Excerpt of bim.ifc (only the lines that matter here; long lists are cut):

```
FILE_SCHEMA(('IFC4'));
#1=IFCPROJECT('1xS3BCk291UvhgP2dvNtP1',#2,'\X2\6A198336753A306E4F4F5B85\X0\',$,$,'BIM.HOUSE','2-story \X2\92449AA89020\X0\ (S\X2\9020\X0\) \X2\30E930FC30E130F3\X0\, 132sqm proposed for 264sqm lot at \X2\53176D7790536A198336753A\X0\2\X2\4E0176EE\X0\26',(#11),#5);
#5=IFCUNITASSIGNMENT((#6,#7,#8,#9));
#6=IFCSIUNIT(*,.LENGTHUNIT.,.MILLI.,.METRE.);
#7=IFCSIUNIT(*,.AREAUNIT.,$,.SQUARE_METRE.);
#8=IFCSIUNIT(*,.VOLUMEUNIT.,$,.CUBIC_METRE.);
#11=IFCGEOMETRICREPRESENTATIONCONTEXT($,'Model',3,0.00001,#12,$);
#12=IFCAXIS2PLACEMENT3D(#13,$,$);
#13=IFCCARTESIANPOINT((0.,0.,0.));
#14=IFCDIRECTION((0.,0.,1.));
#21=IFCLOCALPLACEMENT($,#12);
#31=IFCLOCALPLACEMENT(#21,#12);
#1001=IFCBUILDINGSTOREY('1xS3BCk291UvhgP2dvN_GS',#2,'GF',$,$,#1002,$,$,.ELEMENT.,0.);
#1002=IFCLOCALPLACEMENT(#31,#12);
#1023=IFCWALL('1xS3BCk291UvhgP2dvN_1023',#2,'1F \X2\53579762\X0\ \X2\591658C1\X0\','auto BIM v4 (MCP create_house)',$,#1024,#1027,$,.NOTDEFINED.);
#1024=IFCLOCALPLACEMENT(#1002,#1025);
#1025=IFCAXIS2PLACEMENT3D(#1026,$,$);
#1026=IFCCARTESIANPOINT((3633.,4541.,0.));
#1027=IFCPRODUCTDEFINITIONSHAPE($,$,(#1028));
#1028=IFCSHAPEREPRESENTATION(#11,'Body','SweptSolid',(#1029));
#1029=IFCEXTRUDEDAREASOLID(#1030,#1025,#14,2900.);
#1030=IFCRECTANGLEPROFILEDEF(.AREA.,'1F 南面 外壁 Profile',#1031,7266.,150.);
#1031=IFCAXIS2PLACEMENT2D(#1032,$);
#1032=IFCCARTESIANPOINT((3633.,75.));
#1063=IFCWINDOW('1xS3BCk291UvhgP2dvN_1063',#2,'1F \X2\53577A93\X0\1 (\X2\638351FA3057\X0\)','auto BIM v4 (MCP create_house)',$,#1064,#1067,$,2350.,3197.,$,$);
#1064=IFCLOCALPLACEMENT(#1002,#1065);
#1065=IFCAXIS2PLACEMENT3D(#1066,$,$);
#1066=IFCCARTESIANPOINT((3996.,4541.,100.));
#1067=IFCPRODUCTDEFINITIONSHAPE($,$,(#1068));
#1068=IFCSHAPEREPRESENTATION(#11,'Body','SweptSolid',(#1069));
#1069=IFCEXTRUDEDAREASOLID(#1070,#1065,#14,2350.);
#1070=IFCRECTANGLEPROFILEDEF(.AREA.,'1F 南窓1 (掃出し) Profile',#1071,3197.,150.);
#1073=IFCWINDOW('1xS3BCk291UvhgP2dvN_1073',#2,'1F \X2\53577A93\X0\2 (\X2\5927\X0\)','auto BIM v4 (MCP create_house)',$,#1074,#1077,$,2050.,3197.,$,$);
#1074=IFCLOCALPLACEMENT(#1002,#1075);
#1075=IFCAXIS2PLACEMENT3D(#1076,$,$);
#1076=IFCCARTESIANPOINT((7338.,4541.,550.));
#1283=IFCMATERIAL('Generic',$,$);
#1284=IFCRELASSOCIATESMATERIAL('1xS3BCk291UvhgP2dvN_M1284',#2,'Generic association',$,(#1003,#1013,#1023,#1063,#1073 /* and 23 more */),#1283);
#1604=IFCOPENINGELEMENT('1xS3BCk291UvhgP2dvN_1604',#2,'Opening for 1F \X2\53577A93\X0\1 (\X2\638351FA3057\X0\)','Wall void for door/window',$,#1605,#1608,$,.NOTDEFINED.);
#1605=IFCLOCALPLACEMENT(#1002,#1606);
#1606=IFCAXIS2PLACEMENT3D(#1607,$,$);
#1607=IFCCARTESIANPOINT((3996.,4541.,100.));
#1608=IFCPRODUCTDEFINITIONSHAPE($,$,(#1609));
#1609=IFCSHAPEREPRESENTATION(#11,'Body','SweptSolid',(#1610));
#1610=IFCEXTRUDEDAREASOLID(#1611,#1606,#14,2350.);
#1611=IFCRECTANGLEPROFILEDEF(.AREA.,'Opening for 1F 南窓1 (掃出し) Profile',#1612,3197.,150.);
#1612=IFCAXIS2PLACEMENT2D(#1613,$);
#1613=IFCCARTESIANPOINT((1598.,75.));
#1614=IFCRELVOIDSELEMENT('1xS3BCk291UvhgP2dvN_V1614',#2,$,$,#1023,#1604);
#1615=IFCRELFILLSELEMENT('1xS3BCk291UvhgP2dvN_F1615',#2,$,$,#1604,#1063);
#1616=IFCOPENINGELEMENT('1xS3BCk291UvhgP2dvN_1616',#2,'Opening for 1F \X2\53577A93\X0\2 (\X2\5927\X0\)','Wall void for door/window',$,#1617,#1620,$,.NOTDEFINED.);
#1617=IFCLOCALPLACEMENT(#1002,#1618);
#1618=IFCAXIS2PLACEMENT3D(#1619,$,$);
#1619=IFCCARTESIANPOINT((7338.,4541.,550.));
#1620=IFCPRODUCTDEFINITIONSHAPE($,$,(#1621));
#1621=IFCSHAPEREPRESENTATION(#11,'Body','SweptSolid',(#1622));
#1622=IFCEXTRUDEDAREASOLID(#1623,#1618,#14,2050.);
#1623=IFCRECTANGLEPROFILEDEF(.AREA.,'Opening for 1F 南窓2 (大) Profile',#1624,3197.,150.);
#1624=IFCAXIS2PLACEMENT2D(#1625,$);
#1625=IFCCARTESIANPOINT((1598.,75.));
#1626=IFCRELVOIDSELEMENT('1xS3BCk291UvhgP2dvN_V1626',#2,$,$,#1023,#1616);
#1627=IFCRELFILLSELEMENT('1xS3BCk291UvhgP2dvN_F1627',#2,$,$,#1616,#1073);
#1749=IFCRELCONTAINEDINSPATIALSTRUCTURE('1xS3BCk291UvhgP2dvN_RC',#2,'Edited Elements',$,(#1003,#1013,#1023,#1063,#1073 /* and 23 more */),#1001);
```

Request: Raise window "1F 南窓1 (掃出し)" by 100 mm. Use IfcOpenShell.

```python
import numpy as np
import ifcopenshell
import ifcopenshell.api.geometry
import ifcopenshell.util.placement
import ifcopenshell.util.unit

model = ifcopenshell.open("bim.ifc")
unit_scale = ifcopenshell.util.unit.calculate_unit_scale(model)

window = model.by_guid("1xS3BCk291UvhgP2dvN_1063")
opening = window.FillsVoids[0].RelatingOpeningElement
dz = 0.1 / unit_scale

shift = np.array([0.0, 0.0, dz])
# The window is not placed relative to its opening, so move both.
for product in (opening, window):
    matrix = ifcopenshell.util.placement.get_local_placement(product.ObjectPlacement)
    matrix[:3, 3] += shift
    ifcopenshell.api.geometry.edit_object_placement(model, product=product, matrix=matrix, is_si=False)

print(f"moved by {dz * unit_scale:+.3f} m")

model.write("bim_edited.ifc")
```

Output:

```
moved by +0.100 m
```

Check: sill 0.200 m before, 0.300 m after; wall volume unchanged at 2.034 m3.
